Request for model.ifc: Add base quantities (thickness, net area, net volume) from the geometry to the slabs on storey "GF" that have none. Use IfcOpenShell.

First a look at what the model holds.

```python
import ifcopenshell
import ifcopenshell.util.element
import ifcopenshell.util.unit

model = ifcopenshell.open("model.ifc")
print(model.schema)
for unit_type in ("LENGTHUNIT", "AREAUNIT", "VOLUMEUNIT"):
    print(unit_type, ifcopenshell.util.unit.calculate_unit_scale(model, unit_type))
storey = next(s for s in model.by_type("IfcBuildingStorey") if s.Name == "GF")
slabs = [e for e in ifcopenshell.util.element.get_decomposition(storey) if e.is_a("IfcSlab")]
for e in sorted(slabs, key=lambda e: e.id()):
    print(e.id(), e.is_a(), e.Name, list(ifcopenshell.util.element.get_psets(e, qtos_only=True)), sep=" | ")
```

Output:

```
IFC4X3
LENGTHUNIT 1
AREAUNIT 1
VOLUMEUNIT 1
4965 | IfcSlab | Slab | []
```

```python
import ifcopenshell
import ifcopenshell.api.pset
import ifcopenshell.geom
import ifcopenshell.util.element
import ifcopenshell.util.shape
import ifcopenshell.util.unit

model = ifcopenshell.open("model.ifc")
unit_scale = ifcopenshell.util.unit.calculate_unit_scale(model)
area_scale = ifcopenshell.util.unit.calculate_unit_scale(model, "AREAUNIT")
volume_scale = ifcopenshell.util.unit.calculate_unit_scale(model, "VOLUMEUNIT")
settings = ifcopenshell.geom.settings()

storey = next(s for s in model.by_type("IfcBuildingStorey") if s.Name == "GF")
slabs = [e for e in ifcopenshell.util.element.get_decomposition(storey) if e.is_a("IfcSlab")]

for e in sorted(slabs, key=lambda e: e.id()):
    if ifcopenshell.util.element.get_psets(e, qtos_only=True, should_inherit=False):
        continue
    # Geometry comes back in metres, in the element's own axes.
    shape = ifcopenshell.geom.create_shape(settings, e)
    values = {
        "Width": ifcopenshell.util.shape.get_z(shape.geometry) / unit_scale,
        "NetArea": ifcopenshell.util.shape.get_footprint_area(shape.geometry) / area_scale,
        "NetVolume": ifcopenshell.util.shape.get_volume(shape.geometry) / volume_scale,
    }
    qto = ifcopenshell.api.pset.add_qto(model, product=e, name="Qto_SlabBaseQuantities")
    ifcopenshell.api.pset.edit_qto(model, qto=qto, properties=values)
    print(e.id(), {k: round(v, 3) for k, v in values.items()})

model.write("model-out.ifc")
```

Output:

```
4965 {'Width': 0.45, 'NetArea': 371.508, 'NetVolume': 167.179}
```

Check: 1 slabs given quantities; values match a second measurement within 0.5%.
